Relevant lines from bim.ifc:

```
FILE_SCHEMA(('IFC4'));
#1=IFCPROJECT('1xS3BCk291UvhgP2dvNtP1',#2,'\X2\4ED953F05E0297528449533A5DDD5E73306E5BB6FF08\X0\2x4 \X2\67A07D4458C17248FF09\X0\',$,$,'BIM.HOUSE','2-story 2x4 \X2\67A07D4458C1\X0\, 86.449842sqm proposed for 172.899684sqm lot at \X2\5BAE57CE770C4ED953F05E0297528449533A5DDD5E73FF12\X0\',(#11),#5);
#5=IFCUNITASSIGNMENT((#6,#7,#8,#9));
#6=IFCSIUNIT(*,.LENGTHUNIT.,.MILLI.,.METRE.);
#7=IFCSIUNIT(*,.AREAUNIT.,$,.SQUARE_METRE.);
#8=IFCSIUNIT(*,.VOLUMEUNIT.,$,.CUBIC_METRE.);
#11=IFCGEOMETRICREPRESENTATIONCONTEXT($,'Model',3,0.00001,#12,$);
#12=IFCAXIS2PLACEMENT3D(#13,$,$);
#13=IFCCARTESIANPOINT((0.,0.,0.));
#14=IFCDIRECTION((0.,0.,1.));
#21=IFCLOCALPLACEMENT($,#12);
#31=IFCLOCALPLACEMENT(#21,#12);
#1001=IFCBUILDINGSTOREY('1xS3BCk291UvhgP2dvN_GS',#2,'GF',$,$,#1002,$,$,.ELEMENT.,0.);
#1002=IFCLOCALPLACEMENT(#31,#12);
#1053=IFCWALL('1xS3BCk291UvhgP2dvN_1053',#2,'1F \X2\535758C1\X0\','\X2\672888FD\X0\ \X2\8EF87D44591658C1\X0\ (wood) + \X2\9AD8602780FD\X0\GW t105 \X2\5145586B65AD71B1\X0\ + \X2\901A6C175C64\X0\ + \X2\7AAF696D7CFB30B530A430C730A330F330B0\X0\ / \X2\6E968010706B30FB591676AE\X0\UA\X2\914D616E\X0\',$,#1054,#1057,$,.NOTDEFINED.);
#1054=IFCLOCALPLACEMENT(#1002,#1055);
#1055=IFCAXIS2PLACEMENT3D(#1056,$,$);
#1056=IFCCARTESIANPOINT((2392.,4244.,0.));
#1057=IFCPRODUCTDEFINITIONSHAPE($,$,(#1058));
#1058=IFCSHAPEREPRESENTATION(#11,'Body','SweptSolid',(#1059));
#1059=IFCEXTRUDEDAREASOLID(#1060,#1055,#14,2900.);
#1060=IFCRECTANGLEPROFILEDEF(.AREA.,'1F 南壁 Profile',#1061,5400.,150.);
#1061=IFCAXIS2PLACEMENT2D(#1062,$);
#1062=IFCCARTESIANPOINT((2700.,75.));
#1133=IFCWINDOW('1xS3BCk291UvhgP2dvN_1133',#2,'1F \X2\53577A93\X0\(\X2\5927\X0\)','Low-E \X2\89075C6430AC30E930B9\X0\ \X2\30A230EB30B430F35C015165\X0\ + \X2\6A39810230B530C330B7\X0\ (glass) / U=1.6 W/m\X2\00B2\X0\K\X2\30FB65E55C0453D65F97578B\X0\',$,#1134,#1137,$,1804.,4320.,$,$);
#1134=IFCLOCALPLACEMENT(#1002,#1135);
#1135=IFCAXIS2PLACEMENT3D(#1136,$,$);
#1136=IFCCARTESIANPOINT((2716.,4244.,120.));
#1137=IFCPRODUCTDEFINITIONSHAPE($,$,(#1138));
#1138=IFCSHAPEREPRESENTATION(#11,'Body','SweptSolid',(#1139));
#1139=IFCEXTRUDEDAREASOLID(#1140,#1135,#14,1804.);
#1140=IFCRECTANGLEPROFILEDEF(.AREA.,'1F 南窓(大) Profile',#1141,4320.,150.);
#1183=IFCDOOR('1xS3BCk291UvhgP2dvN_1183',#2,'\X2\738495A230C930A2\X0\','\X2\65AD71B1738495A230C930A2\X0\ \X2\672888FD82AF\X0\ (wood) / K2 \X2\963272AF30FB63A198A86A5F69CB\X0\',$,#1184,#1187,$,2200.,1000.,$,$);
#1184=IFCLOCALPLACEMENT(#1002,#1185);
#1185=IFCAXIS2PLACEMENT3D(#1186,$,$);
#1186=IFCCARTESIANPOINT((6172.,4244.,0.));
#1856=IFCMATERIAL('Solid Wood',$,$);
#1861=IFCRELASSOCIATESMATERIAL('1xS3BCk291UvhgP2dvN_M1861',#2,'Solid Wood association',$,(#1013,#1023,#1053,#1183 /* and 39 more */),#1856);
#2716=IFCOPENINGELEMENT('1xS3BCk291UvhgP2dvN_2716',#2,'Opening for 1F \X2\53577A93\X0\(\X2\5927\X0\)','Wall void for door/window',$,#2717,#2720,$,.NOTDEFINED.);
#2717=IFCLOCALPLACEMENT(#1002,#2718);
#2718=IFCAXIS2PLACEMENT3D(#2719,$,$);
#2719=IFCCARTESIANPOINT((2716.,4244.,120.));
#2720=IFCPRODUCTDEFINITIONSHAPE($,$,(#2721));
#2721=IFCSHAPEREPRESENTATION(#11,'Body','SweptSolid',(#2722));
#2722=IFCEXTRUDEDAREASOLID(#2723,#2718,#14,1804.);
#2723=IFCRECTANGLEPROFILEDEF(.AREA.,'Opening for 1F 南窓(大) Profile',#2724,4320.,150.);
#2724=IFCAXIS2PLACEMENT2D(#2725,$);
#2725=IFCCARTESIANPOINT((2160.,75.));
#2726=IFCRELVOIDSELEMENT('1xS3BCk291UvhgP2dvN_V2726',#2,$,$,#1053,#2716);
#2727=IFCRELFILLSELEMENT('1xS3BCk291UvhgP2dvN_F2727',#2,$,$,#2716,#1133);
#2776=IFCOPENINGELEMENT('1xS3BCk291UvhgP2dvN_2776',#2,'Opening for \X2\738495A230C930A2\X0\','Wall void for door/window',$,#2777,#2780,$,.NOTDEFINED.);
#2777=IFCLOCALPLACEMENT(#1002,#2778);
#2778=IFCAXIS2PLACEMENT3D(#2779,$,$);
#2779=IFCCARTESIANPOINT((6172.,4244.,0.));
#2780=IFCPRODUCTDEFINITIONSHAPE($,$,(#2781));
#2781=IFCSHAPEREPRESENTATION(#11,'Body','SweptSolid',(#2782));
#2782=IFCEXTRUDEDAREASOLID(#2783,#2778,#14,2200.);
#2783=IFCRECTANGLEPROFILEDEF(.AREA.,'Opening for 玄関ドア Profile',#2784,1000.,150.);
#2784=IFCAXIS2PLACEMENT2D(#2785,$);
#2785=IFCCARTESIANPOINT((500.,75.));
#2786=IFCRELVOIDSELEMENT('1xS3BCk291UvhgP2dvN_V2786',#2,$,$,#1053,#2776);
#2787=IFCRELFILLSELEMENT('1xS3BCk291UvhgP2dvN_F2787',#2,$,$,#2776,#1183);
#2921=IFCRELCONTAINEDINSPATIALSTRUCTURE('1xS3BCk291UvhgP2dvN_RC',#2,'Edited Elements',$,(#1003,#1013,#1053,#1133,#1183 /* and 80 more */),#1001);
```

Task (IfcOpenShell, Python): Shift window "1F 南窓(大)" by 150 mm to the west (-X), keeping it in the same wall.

```python
import ifcopenshell
import ifcopenshell.api.geometry
import ifcopenshell.util.placement
import ifcopenshell.util.unit

model = ifcopenshell.open("bim.ifc")
unit_scale = ifcopenshell.util.unit.calculate_unit_scale(model)

window = model.by_guid("1xS3BCk291UvhgP2dvN_1133")
opening = window.FillsVoids[0].RelatingOpeningElement
wall = opening.VoidsElements[0].RelatingBuildingElement

wall_matrix = ifcopenshell.util.placement.get_local_placement(wall.ObjectPlacement)
shift = wall_matrix[:3, 0] * -0.15 / unit_scale
before = ifcopenshell.util.placement.get_local_placement(window.ObjectPlacement)[:3, 3].copy()

# The window is not placed relative to its opening, so move both.
for product in (opening, window):
    matrix = ifcopenshell.util.placement.get_local_placement(product.ObjectPlacement)
    matrix[:3, 3] += shift
    ifcopenshell.api.geometry.edit_object_placement(model, product=product, matrix=matrix, is_si=False)

after = ifcopenshell.util.placement.get_local_placement(window.ObjectPlacement)[:3, 3]
print("window moved by", (after - before).round(3) + 0.0)

model.write("bim_v2.ifc")
```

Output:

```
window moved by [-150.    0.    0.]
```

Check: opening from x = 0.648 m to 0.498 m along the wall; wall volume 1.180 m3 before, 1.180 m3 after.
